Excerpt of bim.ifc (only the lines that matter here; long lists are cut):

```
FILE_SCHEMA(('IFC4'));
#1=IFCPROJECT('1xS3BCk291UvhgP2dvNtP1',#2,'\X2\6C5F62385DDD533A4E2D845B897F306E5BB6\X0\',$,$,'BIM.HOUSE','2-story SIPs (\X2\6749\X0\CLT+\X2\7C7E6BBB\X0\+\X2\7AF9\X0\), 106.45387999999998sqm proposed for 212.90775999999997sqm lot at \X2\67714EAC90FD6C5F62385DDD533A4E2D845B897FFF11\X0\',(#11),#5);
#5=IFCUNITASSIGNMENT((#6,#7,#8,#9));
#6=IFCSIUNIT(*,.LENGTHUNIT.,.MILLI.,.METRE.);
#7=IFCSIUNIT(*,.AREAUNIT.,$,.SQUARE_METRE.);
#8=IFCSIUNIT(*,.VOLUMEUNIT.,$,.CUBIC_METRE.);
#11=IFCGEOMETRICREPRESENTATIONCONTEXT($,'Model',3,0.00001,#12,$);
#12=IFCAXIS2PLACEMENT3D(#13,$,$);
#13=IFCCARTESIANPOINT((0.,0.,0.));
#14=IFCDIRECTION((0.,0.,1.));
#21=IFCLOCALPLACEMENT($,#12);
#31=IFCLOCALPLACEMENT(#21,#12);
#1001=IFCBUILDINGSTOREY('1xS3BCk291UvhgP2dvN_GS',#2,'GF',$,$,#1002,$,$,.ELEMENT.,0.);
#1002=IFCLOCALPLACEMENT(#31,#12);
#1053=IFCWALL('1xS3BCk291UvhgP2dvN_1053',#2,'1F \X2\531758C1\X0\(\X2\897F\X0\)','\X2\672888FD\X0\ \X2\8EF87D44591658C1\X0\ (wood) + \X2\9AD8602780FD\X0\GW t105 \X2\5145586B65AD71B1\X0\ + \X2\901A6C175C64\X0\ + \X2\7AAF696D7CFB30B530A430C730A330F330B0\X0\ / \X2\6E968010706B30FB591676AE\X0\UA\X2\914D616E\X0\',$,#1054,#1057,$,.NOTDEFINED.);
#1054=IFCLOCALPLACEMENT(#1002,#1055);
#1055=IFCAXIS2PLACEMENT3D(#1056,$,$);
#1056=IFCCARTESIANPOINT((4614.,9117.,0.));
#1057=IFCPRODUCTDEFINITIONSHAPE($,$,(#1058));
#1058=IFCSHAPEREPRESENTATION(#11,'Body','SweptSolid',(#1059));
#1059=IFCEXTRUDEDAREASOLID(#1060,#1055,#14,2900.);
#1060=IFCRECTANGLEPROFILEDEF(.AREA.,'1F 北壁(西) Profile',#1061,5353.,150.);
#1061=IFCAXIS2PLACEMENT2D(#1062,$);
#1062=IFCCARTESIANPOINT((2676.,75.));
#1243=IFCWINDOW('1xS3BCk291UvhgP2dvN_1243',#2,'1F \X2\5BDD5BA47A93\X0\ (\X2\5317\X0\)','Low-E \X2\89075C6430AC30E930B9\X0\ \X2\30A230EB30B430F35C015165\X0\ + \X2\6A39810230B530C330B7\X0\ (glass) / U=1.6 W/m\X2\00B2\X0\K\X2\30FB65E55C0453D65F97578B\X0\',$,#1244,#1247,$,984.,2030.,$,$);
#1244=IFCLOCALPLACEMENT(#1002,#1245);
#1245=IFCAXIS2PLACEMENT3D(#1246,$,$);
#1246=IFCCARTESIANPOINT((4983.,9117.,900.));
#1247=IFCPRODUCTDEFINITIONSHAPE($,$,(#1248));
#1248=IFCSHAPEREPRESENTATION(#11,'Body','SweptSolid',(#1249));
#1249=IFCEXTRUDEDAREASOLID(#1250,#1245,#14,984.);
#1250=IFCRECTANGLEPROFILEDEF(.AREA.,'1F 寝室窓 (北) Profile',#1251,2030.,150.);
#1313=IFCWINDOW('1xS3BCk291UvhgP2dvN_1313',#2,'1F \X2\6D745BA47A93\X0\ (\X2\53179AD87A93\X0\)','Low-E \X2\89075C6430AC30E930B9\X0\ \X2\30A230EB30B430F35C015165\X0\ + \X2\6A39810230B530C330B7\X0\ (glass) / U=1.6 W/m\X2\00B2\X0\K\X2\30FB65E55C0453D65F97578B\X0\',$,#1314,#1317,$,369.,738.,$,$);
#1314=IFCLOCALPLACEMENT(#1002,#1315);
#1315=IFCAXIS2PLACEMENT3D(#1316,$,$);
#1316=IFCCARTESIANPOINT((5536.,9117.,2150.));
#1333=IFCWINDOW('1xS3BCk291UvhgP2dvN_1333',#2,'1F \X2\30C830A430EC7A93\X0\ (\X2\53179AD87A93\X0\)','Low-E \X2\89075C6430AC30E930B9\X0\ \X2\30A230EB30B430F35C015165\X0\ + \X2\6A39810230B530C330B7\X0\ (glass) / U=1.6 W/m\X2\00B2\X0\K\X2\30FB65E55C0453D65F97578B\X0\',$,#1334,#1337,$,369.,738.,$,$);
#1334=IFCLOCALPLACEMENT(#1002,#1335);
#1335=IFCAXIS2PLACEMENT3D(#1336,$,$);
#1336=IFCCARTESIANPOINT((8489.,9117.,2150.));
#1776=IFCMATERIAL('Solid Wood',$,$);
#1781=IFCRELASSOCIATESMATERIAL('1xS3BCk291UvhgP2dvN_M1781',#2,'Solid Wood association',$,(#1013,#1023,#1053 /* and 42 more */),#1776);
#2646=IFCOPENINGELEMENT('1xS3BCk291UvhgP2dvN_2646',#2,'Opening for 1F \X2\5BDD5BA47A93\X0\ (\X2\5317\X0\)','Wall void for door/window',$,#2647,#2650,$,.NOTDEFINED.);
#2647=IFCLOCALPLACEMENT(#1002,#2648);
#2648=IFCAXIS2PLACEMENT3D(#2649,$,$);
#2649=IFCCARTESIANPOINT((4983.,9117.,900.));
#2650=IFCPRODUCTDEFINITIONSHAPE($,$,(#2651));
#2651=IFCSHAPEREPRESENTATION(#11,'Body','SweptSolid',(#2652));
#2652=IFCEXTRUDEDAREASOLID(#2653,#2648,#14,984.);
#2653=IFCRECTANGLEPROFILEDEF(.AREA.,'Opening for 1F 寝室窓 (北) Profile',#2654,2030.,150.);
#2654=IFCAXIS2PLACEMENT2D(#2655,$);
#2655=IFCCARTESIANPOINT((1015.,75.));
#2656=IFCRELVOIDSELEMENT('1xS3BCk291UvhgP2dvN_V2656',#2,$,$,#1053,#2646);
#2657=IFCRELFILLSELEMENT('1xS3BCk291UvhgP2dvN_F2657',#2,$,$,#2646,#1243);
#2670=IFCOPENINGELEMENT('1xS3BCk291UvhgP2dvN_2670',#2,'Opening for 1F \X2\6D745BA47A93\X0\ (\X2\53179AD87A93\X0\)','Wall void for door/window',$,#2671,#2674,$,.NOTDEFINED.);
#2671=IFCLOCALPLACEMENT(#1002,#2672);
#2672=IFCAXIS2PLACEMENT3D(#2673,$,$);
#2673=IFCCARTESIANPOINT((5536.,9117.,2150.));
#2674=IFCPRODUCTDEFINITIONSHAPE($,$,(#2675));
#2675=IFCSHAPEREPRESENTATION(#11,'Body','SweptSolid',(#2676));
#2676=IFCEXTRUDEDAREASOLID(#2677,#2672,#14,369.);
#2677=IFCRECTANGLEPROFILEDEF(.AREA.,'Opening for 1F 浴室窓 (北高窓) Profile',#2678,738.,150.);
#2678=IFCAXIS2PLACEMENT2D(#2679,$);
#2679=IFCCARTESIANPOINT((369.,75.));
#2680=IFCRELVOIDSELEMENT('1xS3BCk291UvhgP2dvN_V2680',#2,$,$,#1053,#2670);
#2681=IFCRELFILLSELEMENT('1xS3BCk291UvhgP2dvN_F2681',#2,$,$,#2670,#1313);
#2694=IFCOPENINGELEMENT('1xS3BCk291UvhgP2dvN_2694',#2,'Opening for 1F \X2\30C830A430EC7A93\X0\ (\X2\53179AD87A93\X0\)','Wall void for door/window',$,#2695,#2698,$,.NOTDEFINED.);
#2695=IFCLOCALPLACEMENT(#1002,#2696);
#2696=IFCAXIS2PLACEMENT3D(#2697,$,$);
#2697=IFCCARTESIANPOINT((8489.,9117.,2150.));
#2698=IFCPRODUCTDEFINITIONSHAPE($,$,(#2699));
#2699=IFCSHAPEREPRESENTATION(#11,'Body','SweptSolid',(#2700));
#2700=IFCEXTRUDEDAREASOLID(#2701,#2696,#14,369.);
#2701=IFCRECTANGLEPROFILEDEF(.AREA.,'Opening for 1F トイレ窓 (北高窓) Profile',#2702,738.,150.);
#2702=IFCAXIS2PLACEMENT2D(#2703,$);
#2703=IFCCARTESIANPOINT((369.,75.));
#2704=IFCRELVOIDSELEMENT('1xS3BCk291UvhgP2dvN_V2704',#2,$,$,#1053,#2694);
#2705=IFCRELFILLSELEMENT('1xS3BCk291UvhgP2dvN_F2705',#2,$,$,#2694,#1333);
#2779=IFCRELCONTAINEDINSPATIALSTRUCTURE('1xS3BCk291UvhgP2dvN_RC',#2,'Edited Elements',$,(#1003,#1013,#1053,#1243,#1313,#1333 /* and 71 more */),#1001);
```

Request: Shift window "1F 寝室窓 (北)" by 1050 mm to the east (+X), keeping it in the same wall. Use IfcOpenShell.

```python
import ifcopenshell
import ifcopenshell.api.geometry
import ifcopenshell.util.placement

model = ifcopenshell.open("bim.ifc")

window = model.by_guid("1xS3BCk291UvhgP2dvN_1243")
opening = window.FillsVoids[0].RelatingOpeningElement
wall = opening.VoidsElements[0].RelatingBuildingElement

wall_matrix = ifcopenshell.util.placement.get_local_placement(wall.ObjectPlacement)
shift = wall_matrix[:3, 0] * 1050.0
before = ifcopenshell.util.placement.get_local_placement(window.ObjectPlacement)[:3, 3].copy()

# The window is not placed relative to its opening, so move both.
for product in (opening, window):
    matrix = ifcopenshell.util.placement.get_local_placement(product.ObjectPlacement)
    matrix[:3, 3] += shift
    ifcopenshell.api.geometry.edit_object_placement(model, product=product, matrix=matrix, is_si=False)

after = ifcopenshell.util.placement.get_local_placement(window.ObjectPlacement)[:3, 3]
print("window moved by", (after - before).round(3) + 0.0)

model.write("bim_rev.ifc")
```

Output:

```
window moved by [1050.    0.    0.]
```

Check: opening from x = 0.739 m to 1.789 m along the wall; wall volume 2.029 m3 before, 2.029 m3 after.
